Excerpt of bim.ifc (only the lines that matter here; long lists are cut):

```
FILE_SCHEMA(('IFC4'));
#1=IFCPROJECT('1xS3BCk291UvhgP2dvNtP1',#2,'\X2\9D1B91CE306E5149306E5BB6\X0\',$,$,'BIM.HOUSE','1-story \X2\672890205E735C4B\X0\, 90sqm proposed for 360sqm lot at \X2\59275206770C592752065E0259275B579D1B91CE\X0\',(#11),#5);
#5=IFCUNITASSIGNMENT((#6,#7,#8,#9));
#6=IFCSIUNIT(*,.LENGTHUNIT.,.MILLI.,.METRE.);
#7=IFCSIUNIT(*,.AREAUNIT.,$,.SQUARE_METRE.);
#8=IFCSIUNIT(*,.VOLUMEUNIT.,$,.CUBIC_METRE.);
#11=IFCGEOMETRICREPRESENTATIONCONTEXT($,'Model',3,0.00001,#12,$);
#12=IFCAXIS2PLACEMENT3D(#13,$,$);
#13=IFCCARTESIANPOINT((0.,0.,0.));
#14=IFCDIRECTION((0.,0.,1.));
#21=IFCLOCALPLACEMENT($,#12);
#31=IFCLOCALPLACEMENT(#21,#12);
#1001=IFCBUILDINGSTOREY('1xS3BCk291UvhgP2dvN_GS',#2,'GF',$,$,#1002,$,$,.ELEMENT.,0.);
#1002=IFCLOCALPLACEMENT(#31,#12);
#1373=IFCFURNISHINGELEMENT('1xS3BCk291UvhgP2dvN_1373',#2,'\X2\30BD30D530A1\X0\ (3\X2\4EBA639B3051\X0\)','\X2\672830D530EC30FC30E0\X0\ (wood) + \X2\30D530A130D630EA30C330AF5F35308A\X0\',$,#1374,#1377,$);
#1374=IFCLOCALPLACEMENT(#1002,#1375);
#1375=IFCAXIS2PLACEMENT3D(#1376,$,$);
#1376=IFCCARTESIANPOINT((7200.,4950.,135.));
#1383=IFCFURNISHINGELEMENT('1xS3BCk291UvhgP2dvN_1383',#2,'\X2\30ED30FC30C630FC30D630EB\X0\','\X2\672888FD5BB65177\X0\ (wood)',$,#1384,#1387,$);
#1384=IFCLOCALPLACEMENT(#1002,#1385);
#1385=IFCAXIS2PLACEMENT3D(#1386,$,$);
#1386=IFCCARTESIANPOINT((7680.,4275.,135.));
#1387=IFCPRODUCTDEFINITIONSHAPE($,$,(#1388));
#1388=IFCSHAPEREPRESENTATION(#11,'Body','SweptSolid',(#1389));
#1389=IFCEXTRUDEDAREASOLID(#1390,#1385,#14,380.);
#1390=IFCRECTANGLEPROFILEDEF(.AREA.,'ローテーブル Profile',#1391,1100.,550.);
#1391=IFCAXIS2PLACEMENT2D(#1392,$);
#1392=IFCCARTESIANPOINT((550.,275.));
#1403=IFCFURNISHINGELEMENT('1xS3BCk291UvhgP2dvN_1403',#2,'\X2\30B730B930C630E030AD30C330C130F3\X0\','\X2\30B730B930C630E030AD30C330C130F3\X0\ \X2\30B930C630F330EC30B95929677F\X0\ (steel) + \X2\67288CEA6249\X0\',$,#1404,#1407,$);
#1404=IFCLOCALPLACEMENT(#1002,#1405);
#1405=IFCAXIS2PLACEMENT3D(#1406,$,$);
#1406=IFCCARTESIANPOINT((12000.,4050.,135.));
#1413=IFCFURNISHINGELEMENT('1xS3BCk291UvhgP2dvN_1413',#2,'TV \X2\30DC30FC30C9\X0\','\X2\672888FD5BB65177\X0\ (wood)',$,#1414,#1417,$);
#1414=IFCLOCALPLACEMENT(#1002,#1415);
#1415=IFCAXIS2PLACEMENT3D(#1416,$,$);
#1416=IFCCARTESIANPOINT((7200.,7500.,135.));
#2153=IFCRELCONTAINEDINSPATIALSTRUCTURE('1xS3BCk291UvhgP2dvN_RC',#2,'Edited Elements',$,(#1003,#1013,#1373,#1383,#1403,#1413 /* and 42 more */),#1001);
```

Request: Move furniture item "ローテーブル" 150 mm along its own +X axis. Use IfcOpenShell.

```python
import ifcopenshell
import ifcopenshell.api.geometry
import ifcopenshell.util.placement
import ifcopenshell.util.unit

model = ifcopenshell.open("bim.ifc")
unit_scale = ifcopenshell.util.unit.calculate_unit_scale(model)

item = model.by_id(1383)
matrix = ifcopenshell.util.placement.get_local_placement(item.ObjectPlacement)
matrix[:3, 3] += matrix[:3, 0] * 0.15 / unit_scale
ifcopenshell.api.geometry.edit_object_placement(model, product=item, matrix=matrix, is_si=False)

print(ifcopenshell.util.placement.get_local_placement(item.ObjectPlacement).round(3) + 0.0)

model.write("bim_updated.ifc")
```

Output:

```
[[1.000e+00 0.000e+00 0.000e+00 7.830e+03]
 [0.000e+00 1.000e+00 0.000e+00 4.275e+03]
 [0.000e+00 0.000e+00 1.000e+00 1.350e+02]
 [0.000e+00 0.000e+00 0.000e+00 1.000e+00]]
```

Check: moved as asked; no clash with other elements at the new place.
